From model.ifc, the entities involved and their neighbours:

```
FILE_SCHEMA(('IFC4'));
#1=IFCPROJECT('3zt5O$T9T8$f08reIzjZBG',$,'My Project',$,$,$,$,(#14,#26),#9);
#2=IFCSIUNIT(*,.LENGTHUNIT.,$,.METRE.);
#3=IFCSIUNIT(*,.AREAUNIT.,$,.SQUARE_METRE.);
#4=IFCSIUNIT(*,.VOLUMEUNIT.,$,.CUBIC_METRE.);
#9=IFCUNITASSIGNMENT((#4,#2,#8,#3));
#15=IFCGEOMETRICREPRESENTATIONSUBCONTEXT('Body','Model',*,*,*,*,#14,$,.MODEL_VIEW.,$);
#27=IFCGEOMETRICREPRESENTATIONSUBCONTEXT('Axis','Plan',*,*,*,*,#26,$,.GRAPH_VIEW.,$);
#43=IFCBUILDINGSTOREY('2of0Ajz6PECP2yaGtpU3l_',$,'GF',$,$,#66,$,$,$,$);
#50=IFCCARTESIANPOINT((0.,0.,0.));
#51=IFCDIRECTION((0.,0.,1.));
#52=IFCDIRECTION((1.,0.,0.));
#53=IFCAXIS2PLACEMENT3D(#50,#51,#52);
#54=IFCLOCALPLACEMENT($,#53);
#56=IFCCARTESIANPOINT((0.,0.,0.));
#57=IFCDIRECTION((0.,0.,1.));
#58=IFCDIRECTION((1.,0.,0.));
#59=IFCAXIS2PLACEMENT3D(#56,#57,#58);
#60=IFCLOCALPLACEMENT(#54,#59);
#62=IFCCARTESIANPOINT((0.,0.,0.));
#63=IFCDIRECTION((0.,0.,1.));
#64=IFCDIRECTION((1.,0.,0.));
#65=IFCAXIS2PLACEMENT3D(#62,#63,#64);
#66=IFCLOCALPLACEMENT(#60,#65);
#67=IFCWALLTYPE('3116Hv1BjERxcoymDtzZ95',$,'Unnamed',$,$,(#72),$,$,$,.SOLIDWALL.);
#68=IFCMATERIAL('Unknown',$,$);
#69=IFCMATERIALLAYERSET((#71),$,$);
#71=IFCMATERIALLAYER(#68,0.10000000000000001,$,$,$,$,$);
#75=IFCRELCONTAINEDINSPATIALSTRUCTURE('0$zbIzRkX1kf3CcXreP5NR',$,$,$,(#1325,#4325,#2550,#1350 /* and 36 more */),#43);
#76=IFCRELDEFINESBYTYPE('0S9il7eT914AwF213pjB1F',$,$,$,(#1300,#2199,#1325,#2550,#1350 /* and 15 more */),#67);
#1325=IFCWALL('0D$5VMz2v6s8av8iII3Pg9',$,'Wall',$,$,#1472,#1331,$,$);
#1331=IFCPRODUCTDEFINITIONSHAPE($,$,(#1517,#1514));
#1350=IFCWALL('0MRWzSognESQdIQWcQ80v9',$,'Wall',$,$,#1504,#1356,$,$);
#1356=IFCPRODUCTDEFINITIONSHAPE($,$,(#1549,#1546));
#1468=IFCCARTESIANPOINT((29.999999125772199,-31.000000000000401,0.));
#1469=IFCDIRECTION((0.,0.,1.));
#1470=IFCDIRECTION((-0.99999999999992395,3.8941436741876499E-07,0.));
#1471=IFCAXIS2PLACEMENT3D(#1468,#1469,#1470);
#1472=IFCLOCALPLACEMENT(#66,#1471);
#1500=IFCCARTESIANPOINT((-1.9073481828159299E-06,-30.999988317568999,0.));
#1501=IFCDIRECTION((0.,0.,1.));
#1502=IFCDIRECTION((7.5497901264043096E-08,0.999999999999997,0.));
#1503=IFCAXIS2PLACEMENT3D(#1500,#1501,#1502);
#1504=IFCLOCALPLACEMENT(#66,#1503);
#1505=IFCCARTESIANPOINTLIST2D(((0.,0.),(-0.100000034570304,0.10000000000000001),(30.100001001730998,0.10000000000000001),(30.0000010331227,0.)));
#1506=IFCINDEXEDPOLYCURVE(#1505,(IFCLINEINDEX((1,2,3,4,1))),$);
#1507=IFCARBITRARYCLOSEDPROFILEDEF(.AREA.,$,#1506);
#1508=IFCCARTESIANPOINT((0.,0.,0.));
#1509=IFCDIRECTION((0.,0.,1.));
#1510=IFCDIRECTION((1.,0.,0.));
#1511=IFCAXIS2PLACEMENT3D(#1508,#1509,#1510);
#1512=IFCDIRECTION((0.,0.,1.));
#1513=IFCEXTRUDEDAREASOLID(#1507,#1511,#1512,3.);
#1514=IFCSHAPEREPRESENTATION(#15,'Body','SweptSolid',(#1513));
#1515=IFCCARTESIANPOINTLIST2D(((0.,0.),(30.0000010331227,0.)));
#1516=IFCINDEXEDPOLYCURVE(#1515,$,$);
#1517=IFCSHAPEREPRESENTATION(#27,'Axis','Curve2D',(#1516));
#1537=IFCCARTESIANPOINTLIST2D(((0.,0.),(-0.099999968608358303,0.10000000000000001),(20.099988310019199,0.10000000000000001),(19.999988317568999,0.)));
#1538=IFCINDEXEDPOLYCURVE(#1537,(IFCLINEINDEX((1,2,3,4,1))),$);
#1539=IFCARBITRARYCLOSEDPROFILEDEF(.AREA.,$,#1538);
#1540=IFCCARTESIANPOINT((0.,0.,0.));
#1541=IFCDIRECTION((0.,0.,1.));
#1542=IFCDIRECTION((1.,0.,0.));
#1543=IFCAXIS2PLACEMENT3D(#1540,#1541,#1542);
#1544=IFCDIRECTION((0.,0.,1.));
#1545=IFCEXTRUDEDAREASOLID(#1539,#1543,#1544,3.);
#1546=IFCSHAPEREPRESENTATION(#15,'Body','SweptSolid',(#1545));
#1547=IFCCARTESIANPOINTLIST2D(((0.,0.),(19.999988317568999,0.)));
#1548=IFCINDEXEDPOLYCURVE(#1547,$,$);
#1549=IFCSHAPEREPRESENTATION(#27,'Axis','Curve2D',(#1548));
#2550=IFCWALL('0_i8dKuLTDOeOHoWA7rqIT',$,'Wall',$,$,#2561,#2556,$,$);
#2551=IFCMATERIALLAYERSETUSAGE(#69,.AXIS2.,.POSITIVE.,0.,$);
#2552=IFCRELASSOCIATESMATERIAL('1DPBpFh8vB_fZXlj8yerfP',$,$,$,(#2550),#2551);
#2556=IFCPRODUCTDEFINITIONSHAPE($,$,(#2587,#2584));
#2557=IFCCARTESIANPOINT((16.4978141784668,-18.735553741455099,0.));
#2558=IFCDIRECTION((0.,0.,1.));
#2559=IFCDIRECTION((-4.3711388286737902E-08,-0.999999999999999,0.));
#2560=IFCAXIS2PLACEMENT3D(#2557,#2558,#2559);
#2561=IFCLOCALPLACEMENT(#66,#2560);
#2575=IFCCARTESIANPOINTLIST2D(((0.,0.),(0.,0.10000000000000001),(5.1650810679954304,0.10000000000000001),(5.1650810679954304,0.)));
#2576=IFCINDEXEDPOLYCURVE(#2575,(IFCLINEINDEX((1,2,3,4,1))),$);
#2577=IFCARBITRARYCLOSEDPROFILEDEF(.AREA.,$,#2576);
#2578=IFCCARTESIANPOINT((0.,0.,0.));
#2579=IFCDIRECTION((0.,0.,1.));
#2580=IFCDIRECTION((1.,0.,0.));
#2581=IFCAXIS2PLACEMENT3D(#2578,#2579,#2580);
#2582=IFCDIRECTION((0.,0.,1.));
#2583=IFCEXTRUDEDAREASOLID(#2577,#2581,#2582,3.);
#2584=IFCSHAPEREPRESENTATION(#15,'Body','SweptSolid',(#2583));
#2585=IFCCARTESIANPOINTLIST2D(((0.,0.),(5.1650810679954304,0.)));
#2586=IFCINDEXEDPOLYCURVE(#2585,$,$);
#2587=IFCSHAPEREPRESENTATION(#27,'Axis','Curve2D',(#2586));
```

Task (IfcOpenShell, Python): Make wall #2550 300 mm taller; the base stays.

```python
import ifcopenshell
import ifcopenshell.geom
import ifcopenshell.util.representation
import ifcopenshell.util.shape
import ifcopenshell.util.unit

model = ifcopenshell.open("model.ifc")
unit_scale = ifcopenshell.util.unit.calculate_unit_scale(model)
settings = ifcopenshell.geom.settings()


def volume(element):
    """Net volume in cubic metres, openings subtracted."""
    shape = ifcopenshell.geom.create_shape(settings, element)
    return ifcopenshell.util.shape.get_volume(shape.geometry)


wall = model.by_id(2550)
before = volume(wall)

body = ifcopenshell.util.representation.get_representation(wall, "Model", "Body")
solid = body.Items[0]
old_height = solid.Depth
solid.Depth += 0.3 / unit_scale
after = volume(wall)

print(f"height {old_height:g} -> {solid.Depth:g}, volume {before:.3f} -> {after:.3f} m3")

model.write("model_rev.ifc")
```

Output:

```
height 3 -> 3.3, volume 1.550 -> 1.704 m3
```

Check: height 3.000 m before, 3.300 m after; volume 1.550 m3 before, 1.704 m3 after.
